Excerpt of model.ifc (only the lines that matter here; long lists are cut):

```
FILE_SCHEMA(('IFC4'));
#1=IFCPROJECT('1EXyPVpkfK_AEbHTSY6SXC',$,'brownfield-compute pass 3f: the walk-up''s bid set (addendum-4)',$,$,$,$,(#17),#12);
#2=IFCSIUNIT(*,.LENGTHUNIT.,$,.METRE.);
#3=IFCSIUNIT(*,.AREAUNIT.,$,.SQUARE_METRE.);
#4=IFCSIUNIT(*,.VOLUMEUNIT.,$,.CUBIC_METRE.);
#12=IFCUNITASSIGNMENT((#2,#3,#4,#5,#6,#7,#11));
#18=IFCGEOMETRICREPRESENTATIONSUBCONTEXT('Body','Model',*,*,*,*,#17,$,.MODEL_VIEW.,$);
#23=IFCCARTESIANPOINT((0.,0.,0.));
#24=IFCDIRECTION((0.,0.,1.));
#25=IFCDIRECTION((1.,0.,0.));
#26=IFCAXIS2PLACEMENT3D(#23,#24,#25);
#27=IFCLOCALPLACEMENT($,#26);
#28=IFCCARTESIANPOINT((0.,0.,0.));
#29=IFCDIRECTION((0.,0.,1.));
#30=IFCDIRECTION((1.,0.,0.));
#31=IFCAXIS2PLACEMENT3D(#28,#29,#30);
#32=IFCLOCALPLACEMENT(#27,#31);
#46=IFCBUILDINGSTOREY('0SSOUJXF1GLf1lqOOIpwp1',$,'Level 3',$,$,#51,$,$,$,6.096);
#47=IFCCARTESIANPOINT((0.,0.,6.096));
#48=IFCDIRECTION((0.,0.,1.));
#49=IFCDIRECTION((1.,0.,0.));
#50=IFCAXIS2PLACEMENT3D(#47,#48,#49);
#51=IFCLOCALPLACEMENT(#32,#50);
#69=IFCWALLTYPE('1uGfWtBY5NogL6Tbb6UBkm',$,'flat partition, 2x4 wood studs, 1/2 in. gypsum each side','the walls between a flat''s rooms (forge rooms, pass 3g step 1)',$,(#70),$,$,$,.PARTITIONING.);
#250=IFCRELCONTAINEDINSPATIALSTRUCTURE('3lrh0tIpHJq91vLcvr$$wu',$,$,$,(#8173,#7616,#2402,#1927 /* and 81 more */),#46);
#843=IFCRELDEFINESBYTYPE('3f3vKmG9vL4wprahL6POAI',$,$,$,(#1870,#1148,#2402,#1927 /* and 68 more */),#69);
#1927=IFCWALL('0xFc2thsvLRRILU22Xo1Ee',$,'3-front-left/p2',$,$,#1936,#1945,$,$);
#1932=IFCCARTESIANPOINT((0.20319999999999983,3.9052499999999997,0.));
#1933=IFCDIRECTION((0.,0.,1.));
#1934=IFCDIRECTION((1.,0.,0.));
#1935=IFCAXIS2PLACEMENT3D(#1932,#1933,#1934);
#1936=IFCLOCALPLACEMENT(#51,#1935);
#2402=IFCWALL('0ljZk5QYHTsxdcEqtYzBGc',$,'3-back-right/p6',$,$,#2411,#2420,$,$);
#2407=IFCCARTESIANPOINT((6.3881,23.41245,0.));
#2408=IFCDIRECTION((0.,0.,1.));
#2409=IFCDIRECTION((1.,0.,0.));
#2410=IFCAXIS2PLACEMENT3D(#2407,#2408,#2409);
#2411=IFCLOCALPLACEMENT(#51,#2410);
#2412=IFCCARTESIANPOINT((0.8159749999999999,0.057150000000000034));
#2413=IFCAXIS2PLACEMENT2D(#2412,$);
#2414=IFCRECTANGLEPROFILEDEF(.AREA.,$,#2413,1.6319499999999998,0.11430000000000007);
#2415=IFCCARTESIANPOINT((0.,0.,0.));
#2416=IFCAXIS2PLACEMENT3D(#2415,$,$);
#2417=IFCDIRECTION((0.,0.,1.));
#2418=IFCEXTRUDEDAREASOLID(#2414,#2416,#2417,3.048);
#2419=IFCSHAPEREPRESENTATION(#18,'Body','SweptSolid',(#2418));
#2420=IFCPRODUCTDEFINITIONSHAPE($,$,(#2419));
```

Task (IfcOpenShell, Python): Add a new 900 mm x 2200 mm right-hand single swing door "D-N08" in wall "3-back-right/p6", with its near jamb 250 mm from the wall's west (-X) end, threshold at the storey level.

```python
import numpy as np
import ifcopenshell
import ifcopenshell.api.feature
import ifcopenshell.api.geometry
import ifcopenshell.api.root
import ifcopenshell.api.spatial
import ifcopenshell.geom
import ifcopenshell.util.element
import ifcopenshell.util.placement
import ifcopenshell.util.representation
import ifcopenshell.util.shape
import ifcopenshell.util.unit

model = ifcopenshell.open("model.ifc")
unit_scale = ifcopenshell.util.unit.calculate_unit_scale(model)
settings = ifcopenshell.geom.settings()


def volume(element):
    """Net volume in cubic metres, openings subtracted."""
    shape = ifcopenshell.geom.create_shape(settings, element)
    return ifcopenshell.util.shape.get_volume(shape.geometry)


wall = model.by_guid("0ljZk5QYHTsxdcEqtYzBGc")
storey = ifcopenshell.util.element.get_container(wall, ifc_class="IfcBuildingStorey")
context = ifcopenshell.util.representation.get_context(model, "Model", "Body", "MODEL_VIEW")
before = volume(wall)

width, height, from_end, sill = 0.9, 2.2, 0.25, 0.0  # metres

# The wall runs along its own X axis, and the end named is its -X end.
wall_shape = ifcopenshell.geom.create_shape(settings, wall)
x, y, z = ifcopenshell.util.shape.get_vertices(wall_shape.geometry).T
start = x.min() + from_end
face, thickness = float(y.min()), float(y.max() - y.min())
wall_matrix = ifcopenshell.util.placement.get_local_placement(wall.ObjectPlacement)
level = ifcopenshell.util.placement.get_local_placement(storey.ObjectPlacement)[2, 3]


def in_wall(x, y):
    """Placement at x, y metres in the wall's axes, at sill height."""
    matrix = wall_matrix.copy()
    matrix[:, 3] = wall_matrix @ np.array([x / unit_scale, y / unit_scale, 0.0, 1.0])
    matrix[2, 3] = level + sill / unit_scale
    return matrix


# Opening: a box that overshoots both wall faces by 50 mm.
opening = ifcopenshell.api.root.create_entity(model, ifc_class="IfcOpeningElement", predefined_type="OPENING")
box = ifcopenshell.api.geometry.add_wall_representation(
    model, context=context, length=width, height=height, thickness=thickness + 0.1
)
ifcopenshell.api.geometry.assign_representation(model, product=opening, representation=box)
ifcopenshell.api.geometry.edit_object_placement(model, product=opening, matrix=in_wall(start, face - 0.05), is_si=False)
ifcopenshell.api.feature.add_feature(model, feature=opening, element=wall)

door = ifcopenshell.api.root.create_entity(model, ifc_class="IfcDoor", name="D-N08", predefined_type="DOOR")
door.OverallWidth, door.OverallHeight = width / unit_scale, height / unit_scale
door.OperationType = "SINGLE_SWING_RIGHT"
body = ifcopenshell.api.geometry.add_door_representation(
    model,
    context=context,
    overall_width=door.OverallWidth,
    overall_height=door.OverallHeight,
    operation_type="SINGLE_SWING_RIGHT",
    lining_properties={"LiningDepth": thickness / unit_scale, "ThresholdDepth": thickness / unit_scale},
)
ifcopenshell.api.geometry.assign_representation(model, product=door, representation=body)
ifcopenshell.api.spatial.assign_container(model, products=[door], relating_structure=storey)
ifcopenshell.api.feature.add_filling(model, opening=opening, element=door)

# The lining spans the wall, so the door starts at the wall face.
ifcopenshell.api.geometry.edit_object_placement(model, product=door, matrix=in_wall(start, face), is_si=False)

after = volume(wall)

print(f"wall volume {before:.3f} -> {after:.3f} m3")

model.write("model_edited.ifc")
```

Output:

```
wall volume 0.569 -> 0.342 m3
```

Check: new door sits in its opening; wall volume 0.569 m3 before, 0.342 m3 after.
